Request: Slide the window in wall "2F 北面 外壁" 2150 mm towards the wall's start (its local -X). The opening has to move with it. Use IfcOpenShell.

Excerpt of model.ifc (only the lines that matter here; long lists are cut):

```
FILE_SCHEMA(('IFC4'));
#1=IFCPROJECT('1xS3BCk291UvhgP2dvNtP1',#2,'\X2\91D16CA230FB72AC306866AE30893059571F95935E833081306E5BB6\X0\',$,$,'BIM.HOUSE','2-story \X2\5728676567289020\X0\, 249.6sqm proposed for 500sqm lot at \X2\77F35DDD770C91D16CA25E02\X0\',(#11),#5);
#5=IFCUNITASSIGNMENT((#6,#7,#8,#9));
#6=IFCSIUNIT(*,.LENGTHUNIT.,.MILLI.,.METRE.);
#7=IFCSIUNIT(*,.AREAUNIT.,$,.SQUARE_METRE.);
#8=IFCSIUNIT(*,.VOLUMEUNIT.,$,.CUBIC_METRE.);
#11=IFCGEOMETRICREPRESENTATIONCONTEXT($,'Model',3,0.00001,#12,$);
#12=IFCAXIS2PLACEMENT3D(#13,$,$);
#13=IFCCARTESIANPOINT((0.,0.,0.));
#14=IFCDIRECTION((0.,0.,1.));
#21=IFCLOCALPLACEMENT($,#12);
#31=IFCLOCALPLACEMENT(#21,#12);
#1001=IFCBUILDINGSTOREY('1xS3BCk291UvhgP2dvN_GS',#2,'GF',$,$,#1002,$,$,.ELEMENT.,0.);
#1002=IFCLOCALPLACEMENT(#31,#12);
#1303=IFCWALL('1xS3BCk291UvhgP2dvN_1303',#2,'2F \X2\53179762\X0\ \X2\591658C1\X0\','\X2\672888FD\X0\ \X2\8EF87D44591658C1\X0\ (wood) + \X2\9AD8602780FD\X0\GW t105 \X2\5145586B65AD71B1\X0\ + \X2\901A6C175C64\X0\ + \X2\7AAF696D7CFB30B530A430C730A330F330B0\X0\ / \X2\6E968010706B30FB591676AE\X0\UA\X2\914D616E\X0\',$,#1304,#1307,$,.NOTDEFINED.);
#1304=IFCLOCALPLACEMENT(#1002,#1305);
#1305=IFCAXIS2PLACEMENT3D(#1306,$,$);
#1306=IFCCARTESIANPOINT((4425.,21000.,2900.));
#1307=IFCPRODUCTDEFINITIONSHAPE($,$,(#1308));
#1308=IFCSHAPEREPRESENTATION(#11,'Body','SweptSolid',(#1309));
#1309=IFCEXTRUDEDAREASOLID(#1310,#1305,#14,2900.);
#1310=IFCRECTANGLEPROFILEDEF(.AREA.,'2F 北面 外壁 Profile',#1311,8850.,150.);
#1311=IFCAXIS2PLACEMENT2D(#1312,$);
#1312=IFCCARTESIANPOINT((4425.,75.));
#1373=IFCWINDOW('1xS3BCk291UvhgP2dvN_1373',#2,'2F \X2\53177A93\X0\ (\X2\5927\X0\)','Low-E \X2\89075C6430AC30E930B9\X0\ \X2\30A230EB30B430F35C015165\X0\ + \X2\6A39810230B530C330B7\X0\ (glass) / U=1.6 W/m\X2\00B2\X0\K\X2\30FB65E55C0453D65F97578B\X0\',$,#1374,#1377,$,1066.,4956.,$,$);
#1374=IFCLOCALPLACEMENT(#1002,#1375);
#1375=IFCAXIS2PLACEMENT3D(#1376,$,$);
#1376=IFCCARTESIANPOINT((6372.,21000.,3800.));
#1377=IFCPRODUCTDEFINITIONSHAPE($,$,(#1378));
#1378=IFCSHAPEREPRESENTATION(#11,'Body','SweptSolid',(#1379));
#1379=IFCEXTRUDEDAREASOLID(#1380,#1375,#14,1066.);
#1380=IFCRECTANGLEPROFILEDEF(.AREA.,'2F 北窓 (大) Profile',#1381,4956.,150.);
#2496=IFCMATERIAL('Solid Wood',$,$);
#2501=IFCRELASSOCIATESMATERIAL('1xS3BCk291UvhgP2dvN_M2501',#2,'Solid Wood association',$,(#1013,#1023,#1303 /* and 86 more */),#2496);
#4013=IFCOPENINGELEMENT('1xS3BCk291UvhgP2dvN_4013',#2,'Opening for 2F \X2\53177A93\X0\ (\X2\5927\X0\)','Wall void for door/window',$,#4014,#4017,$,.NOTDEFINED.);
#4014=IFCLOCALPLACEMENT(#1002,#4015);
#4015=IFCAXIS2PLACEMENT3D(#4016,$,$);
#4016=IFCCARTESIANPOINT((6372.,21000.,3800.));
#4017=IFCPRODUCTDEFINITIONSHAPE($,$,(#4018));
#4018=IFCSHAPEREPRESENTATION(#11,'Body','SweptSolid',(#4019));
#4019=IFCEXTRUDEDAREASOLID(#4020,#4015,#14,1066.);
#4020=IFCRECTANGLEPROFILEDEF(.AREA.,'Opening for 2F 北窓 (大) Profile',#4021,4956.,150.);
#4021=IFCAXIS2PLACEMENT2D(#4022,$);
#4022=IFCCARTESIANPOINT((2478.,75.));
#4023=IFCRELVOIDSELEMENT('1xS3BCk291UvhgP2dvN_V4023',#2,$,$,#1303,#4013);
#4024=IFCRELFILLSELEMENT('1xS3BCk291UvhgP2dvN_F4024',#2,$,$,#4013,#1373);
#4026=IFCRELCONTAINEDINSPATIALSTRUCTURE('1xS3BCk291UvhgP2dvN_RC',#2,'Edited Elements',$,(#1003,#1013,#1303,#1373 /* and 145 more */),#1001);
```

```python
import ifcopenshell
import ifcopenshell.api.geometry
import ifcopenshell.util.placement

model = ifcopenshell.open("model.ifc")

window = model.by_guid("1xS3BCk291UvhgP2dvN_1373")
opening = window.FillsVoids[0].RelatingOpeningElement
wall = opening.VoidsElements[0].RelatingBuildingElement

wall_matrix = ifcopenshell.util.placement.get_local_placement(wall.ObjectPlacement)
shift = wall_matrix[:3, 0] * -2150.0
before = ifcopenshell.util.placement.get_local_placement(window.ObjectPlacement)[:3, 3].copy()

# The window is not placed relative to its opening, so move both.
for product in (opening, window):
    matrix = ifcopenshell.util.placement.get_local_placement(product.ObjectPlacement)
    matrix[:3, 3] += shift
    ifcopenshell.api.geometry.edit_object_placement(model, product=product, matrix=matrix, is_si=False)

after = ifcopenshell.util.placement.get_local_placement(window.ObjectPlacement)[:3, 3]
print("window moved by", (after - before).round(3) + 0.0)

model.write("model_updated.ifc")
```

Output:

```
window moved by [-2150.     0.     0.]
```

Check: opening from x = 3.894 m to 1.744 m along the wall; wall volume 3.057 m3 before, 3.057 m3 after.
